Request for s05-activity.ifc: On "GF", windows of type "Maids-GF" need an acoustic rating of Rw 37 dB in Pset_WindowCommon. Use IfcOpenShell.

First a look at what the model holds.

```python
import ifcopenshell
import ifcopenshell.util.element

model = ifcopenshell.open("s05-activity.ifc")
print(model.schema)
storey = next(s for s in model.by_type("IfcBuildingStorey") if s.Name == "GF")
windows = [e for e in ifcopenshell.util.element.get_decomposition(storey) if e.is_a("IfcWindow")]
seen = {}
for e in windows:
    element_type = ifcopenshell.util.element.get_type(e)
    key = (element_type.Name if element_type != e and element_type else None, ifcopenshell.util.element.get_pset(e, "Pset_WindowCommon", "AcousticRating"))
    seen[key] = seen.get(key, 0) + 1
for (name, value), count in sorted(seen.items(), key=str):
    print(count, "x", name, "|", value)
```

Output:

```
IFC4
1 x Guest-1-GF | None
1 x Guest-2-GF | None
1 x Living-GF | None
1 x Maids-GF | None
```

```python
import ifcopenshell
import ifcopenshell.api.pset
import ifcopenshell.util.element

model = ifcopenshell.open("s05-activity.ifc")

storey = next(s for s in model.by_type("IfcBuildingStorey") if s.Name == "GF")
windows = [e for e in ifcopenshell.util.element.get_decomposition(storey) if e.is_a("IfcWindow")]

count = 0
for e in windows:
    element_type = ifcopenshell.util.element.get_type(e)
    if element_type in (None, e) or element_type.Name != "Maids-GF":
        continue
    # add_pset returns the element's existing set when there is one.
    pset = ifcopenshell.api.pset.add_pset(model, product=e, name="Pset_WindowCommon")
    ifcopenshell.api.pset.edit_pset(model, pset=pset, properties={"AcousticRating": "Rw 37 dB"})
    count += 1

print(count, "windows updated")

model.write("s05-activity_rev.ifc")
```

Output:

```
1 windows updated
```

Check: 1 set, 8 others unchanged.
